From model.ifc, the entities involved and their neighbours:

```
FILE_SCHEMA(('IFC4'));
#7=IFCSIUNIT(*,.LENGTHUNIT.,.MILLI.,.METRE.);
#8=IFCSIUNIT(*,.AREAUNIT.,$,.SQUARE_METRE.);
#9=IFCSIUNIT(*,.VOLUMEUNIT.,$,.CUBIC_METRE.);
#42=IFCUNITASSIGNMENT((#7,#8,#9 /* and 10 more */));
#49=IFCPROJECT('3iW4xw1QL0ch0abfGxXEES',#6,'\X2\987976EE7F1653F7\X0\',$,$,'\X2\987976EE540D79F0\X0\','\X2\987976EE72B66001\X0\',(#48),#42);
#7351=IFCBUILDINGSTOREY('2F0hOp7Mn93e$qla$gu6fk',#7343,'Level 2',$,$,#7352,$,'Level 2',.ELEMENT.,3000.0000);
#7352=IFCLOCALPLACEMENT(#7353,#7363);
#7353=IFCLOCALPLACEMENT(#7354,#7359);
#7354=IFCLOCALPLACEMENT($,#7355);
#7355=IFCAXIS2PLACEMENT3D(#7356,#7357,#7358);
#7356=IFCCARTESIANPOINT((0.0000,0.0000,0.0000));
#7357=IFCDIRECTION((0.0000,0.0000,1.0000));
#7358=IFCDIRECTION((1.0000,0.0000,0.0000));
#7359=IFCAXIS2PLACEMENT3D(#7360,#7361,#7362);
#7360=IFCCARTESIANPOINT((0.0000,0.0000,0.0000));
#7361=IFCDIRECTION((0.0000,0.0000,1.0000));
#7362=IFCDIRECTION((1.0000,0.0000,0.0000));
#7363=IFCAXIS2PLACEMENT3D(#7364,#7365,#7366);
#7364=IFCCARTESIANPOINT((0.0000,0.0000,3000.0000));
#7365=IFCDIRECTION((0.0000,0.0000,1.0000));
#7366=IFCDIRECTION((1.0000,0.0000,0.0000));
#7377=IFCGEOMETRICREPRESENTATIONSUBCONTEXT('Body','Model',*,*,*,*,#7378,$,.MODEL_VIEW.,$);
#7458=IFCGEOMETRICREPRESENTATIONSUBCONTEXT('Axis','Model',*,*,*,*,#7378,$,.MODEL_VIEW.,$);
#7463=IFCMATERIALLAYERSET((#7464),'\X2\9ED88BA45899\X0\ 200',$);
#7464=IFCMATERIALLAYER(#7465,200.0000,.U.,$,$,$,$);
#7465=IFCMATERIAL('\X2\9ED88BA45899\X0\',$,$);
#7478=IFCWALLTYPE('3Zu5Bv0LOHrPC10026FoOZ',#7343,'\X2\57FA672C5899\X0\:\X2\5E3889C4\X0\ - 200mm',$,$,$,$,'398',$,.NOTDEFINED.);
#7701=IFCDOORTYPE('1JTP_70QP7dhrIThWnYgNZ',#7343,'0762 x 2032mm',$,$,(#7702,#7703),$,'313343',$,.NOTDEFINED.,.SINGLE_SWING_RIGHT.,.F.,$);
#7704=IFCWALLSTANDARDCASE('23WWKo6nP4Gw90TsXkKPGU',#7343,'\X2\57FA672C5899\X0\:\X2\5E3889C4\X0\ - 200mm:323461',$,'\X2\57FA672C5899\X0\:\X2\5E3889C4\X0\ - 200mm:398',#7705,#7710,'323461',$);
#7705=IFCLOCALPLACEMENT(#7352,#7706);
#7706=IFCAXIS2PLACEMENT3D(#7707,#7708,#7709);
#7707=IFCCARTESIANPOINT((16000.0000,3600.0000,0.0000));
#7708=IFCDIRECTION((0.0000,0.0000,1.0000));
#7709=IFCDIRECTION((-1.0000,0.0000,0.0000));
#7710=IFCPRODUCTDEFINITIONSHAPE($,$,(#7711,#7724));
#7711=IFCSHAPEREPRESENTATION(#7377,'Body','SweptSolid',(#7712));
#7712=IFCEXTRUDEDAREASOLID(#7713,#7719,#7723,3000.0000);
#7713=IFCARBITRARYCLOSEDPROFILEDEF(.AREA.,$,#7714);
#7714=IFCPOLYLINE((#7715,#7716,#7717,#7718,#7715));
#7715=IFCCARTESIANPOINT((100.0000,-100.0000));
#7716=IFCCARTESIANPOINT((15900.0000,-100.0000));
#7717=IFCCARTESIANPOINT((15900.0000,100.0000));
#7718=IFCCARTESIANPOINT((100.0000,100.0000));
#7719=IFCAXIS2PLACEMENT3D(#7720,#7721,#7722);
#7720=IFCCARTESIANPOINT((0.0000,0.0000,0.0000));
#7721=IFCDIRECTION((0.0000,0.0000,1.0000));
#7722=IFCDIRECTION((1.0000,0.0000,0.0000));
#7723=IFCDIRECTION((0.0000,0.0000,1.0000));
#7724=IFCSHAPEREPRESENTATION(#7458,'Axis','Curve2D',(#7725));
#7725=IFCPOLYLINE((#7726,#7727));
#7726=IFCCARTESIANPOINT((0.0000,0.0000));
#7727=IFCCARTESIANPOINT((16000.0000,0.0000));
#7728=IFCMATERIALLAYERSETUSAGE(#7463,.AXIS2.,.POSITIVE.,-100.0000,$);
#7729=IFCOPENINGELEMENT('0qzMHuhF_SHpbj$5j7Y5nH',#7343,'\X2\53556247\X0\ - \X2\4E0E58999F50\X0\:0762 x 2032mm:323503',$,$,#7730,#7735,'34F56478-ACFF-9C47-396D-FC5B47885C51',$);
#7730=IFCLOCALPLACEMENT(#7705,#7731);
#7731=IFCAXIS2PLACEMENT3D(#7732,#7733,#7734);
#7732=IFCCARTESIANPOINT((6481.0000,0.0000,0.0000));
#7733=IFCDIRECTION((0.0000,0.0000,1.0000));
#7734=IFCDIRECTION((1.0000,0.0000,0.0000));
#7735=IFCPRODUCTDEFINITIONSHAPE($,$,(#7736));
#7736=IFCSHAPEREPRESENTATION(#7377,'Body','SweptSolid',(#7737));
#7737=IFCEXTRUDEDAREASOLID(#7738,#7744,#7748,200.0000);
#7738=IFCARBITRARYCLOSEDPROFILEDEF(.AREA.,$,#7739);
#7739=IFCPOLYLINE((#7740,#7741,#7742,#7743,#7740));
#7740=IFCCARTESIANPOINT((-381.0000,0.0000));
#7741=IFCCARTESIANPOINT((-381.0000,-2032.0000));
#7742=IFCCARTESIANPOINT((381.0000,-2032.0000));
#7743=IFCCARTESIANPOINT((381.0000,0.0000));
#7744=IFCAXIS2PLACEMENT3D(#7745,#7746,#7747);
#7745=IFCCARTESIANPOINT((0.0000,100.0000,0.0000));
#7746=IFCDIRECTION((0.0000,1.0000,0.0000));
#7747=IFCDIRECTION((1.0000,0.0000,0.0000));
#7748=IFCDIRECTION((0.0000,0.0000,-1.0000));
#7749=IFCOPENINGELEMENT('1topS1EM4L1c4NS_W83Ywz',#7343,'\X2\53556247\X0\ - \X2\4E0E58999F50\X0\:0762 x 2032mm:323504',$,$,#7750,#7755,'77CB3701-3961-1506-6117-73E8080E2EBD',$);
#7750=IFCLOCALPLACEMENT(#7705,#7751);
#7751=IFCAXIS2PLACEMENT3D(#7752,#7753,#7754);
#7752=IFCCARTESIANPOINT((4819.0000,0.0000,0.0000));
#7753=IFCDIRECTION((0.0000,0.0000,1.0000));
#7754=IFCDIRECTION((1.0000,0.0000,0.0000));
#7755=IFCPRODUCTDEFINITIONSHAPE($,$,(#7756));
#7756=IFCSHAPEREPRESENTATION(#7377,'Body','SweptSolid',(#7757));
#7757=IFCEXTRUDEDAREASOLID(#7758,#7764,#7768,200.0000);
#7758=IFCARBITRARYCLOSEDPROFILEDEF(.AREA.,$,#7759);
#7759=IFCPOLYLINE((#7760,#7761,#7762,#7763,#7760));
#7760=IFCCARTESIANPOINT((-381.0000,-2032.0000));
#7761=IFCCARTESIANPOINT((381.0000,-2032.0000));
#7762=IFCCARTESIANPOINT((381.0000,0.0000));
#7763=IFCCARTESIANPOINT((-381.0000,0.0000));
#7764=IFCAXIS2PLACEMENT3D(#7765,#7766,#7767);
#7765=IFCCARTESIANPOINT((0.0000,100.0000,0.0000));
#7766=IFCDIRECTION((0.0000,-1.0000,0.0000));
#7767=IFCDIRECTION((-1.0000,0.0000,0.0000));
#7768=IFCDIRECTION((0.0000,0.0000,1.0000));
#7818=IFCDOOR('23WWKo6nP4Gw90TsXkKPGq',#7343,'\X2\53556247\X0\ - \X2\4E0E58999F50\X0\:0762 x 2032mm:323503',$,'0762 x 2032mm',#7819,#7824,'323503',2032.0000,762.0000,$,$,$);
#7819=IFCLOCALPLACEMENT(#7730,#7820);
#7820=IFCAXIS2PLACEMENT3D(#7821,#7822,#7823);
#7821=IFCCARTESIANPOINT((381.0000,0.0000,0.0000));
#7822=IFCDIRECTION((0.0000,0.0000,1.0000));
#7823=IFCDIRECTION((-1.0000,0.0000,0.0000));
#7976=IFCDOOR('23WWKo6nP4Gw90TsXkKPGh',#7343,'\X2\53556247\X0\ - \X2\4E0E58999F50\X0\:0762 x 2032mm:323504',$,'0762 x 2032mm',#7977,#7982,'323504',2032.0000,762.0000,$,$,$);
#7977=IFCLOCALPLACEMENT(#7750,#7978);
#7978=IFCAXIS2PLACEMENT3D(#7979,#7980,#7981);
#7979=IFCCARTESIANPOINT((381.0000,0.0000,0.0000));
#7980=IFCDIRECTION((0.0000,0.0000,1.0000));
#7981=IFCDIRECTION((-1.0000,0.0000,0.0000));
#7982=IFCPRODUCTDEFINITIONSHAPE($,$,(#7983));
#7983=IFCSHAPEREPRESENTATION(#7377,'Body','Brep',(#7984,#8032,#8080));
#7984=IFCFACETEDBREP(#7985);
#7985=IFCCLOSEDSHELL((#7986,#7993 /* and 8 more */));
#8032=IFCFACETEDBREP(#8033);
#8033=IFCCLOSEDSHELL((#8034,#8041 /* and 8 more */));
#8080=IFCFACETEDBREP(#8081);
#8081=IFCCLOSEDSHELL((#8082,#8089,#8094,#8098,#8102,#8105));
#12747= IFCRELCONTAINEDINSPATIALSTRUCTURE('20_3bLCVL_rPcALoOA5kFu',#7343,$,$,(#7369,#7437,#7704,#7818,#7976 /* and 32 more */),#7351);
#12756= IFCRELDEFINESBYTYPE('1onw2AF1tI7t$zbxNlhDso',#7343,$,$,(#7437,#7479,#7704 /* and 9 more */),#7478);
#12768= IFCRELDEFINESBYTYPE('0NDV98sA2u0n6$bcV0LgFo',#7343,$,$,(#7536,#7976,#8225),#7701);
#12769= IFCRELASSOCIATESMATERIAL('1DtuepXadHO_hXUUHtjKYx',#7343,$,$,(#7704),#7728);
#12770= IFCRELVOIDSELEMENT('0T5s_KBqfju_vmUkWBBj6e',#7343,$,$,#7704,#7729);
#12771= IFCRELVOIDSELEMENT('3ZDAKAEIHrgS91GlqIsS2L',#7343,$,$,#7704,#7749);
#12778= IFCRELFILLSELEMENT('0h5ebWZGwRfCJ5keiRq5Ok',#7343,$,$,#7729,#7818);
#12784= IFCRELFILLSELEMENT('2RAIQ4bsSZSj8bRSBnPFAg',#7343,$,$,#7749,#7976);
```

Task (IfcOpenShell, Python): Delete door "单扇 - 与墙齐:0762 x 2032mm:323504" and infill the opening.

```python
import ifcopenshell
import ifcopenshell.api.feature
import ifcopenshell.api.root
import ifcopenshell.geom
import ifcopenshell.util.shape

model = ifcopenshell.open("model.ifc")
settings = ifcopenshell.geom.settings()


def volume(element):
    """Net volume in cubic metres, openings subtracted."""
    shape = ifcopenshell.geom.create_shape(settings, element)
    return ifcopenshell.util.shape.get_volume(shape.geometry)


door = model.by_guid("23WWKo6nP4Gw90TsXkKPGh")
opening = door.FillsVoids[0].RelatingOpeningElement
wall = opening.VoidsElements[0].RelatingBuildingElement
before = volume(wall)

ifcopenshell.api.root.remove_product(model, product=door)
ifcopenshell.api.feature.remove_feature(model, feature=opening)

after = volume(wall)

print(f"wall volume {before:.3f} -> {after:.3f} m3")

model.write("model_edited.ifc")
```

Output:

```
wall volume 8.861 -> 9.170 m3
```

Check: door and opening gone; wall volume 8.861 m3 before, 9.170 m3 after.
